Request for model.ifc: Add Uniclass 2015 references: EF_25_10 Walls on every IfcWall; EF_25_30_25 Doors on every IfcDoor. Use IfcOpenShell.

First a look at what the model holds.

```python
import ifcopenshell

model = ifcopenshell.open("model.ifc")
print(model.schema)
print("classifications:", [c.Name for c in model.by_type("IfcClassification")])
for ifc_class in ("IfcDoor", "IfcRoof", "IfcStair", "IfcWall", "IfcWindow"):
    print(ifc_class, len(model.by_type(ifc_class)))
```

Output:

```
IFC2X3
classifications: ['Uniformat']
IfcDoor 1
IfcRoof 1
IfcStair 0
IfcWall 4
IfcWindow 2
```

```python
import ifcopenshell
import ifcopenshell.api.classification

model = ifcopenshell.open("model.ifc")

# IFC2X3 requires Source and Edition and has no link from the project to the system.
system = model.create_entity("IfcClassification", Source="NBS", Edition="2015", Name="Uniclass 2015")

codes = {
    "IfcWall": ("EF_25_10", "Walls"),
    "IfcDoor": ("EF_25_30_25", "Doors"),
}
for ifc_class, (code, name) in codes.items():
    products = model.by_type(ifc_class)
    ifcopenshell.api.classification.add_reference(
        model, products=products, classification=system, identification=code, name=name
    )
    print(code, len(products))

model.write("model_rev.ifc")
```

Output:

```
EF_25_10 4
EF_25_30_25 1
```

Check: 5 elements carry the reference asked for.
